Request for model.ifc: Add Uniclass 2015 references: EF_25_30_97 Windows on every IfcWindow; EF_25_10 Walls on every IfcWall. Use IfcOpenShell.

First a look at what the model holds.

```python
import ifcopenshell

model = ifcopenshell.open("model.ifc")
print(model.schema)
print("classifications:", [c.Name for c in model.by_type("IfcClassification")])
for ifc_class in ("IfcDoor", "IfcRoof", "IfcStair", "IfcWall", "IfcWindow"):
    print(ifc_class, len(model.by_type(ifc_class)))
```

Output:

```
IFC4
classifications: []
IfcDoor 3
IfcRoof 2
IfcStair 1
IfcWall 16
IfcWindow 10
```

```python
import ifcopenshell
import ifcopenshell.api.classification

model = ifcopenshell.open("model.ifc")

system = ifcopenshell.api.classification.add_classification(model, classification="Uniclass 2015")

codes = {
    "IfcWindow": ("EF_25_30_97", "Windows"),
    "IfcWall": ("EF_25_10", "Walls"),
}
for ifc_class, (code, name) in codes.items():
    products = model.by_type(ifc_class)
    ifcopenshell.api.classification.add_reference(
        model, products=products, classification=system, identification=code, name=name
    )
    print(code, len(products))

model.write("model_v2.ifc")
```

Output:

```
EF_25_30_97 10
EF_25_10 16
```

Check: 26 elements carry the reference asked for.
